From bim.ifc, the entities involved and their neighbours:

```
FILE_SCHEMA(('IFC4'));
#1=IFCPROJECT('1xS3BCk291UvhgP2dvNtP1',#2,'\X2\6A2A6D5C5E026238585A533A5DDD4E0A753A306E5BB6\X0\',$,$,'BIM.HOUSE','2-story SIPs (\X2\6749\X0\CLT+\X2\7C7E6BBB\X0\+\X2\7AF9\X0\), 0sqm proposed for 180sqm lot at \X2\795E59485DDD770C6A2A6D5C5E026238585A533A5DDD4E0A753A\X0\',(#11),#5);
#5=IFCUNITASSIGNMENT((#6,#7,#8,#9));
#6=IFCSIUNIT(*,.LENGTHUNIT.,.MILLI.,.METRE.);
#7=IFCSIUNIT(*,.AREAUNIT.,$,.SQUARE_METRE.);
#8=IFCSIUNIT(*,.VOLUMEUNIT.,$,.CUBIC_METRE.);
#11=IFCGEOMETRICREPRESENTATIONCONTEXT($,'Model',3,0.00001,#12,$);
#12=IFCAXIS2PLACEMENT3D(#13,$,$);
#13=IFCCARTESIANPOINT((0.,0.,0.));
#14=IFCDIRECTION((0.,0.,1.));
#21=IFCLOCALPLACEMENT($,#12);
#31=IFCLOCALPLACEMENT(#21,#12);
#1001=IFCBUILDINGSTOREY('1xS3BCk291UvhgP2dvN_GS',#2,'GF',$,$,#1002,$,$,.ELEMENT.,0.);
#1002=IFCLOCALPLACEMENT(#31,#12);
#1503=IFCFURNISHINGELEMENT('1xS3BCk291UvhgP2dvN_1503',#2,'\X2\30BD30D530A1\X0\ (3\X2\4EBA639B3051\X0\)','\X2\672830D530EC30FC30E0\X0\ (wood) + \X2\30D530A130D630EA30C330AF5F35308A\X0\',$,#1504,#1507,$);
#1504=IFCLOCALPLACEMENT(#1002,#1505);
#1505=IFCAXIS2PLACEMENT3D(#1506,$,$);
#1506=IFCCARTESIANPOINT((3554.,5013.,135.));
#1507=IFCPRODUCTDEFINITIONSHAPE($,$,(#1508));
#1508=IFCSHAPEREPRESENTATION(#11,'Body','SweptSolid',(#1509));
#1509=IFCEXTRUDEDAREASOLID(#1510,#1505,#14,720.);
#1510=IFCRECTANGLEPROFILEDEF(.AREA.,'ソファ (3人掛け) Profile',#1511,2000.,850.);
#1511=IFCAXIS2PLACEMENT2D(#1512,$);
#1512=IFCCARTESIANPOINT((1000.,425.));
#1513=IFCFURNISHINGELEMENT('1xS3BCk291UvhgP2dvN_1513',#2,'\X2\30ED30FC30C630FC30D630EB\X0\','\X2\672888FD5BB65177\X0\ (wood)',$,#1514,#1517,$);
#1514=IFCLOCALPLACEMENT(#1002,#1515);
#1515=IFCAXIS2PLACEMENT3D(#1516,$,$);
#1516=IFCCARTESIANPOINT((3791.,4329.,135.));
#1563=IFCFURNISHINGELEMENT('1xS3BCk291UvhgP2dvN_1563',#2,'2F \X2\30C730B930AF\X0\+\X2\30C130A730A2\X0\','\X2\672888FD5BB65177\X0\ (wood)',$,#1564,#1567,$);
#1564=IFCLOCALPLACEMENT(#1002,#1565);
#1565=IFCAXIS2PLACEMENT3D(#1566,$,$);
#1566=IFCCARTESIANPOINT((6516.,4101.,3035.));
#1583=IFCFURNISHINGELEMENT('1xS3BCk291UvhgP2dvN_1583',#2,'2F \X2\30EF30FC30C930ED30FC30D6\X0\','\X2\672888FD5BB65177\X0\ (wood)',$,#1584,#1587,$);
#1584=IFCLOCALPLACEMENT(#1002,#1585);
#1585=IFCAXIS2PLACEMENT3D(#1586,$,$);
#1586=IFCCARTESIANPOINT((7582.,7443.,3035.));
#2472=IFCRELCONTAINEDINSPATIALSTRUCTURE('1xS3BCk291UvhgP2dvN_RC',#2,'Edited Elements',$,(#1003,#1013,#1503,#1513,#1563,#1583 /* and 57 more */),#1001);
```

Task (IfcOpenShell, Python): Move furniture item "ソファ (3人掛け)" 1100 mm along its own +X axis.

```python
import ifcopenshell
import ifcopenshell.api.geometry
import ifcopenshell.util.placement
import ifcopenshell.util.unit

model = ifcopenshell.open("bim.ifc")
unit_scale = ifcopenshell.util.unit.calculate_unit_scale(model)

item = model.by_guid("1xS3BCk291UvhgP2dvN_1503")
matrix = ifcopenshell.util.placement.get_local_placement(item.ObjectPlacement)
matrix[:3, 3] += matrix[:3, 0] * 1.1 / unit_scale
ifcopenshell.api.geometry.edit_object_placement(model, product=item, matrix=matrix, is_si=False)

print(ifcopenshell.util.placement.get_local_placement(item.ObjectPlacement).round(3) + 0.0)

model.write("bim_v2.ifc")
```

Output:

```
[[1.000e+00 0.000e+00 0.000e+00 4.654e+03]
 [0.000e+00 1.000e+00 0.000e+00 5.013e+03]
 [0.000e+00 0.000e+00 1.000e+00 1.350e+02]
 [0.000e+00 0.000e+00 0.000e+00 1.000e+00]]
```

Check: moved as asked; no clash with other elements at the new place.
